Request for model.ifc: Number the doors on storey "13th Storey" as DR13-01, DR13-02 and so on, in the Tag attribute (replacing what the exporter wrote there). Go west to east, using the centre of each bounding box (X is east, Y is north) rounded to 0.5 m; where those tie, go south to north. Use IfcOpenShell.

First a look at what the model holds.

```python
import ifcopenshell
import ifcopenshell.util.element
import ifcopenshell.util.placement

model = ifcopenshell.open("model.ifc")
print(model.schema)
storey = next(s for s in model.by_type("IfcBuildingStorey") if s.Name == "13th Storey")
doors = [e for e in ifcopenshell.util.element.get_decomposition(storey) if e.is_a("IfcDoor")]
for e in sorted(doors, key=lambda e: e.id()):
    origin = ifcopenshell.util.placement.get_local_placement(e.ObjectPlacement)[:3, 3]
    print(e.id(), e.Tag, e.Name, origin.round(2) + 0.0, sep=" | ")
```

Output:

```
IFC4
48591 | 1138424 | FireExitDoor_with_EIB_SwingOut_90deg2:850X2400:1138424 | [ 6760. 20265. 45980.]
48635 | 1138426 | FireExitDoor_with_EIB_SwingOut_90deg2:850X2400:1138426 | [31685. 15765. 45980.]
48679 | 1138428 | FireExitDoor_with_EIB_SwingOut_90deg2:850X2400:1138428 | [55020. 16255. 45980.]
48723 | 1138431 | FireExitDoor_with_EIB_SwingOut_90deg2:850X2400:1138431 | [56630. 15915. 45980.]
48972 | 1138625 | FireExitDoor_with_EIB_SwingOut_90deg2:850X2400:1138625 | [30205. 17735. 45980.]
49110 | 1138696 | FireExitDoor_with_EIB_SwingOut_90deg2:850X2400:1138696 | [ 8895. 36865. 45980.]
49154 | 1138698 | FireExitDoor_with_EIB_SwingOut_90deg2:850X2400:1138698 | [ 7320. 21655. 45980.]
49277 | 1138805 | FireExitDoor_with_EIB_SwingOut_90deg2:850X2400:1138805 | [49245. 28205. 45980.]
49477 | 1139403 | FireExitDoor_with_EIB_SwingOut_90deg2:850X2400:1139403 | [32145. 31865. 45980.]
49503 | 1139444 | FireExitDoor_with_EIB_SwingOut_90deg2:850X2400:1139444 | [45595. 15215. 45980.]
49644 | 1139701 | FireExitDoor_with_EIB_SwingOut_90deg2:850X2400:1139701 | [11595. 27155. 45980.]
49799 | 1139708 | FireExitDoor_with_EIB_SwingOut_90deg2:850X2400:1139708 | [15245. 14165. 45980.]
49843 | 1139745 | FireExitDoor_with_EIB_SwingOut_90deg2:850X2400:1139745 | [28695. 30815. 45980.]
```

```python
import ifcopenshell
import ifcopenshell.geom
import ifcopenshell.util.element
import ifcopenshell.util.shape

model = ifcopenshell.open("model.ifc")
settings = ifcopenshell.geom.settings()
settings.set("use-world-coords", True)


def centre(element):
    shape = ifcopenshell.geom.create_shape(settings, element)
    return ifcopenshell.util.shape.get_bbox_centroid(shape.geometry)


storey = next(s for s in model.by_type("IfcBuildingStorey") if s.Name == "13th Storey")
doors = [e for e in ifcopenshell.util.element.get_decomposition(storey) if e.is_a("IfcDoor")]

# Insertion points can sit at a corner or the storey origin, so sort by the geometry (in metres).
centres = {e: centre(e) for e in doors}
doors.sort(key=lambda e: (round(centres[e][0] / 0.5), centres[e][1]))

for i, e in enumerate(doors, start=1):
    number = f"DR13-{i:02d}"
    e.Tag = number
    print(e.id(), number)

model.write("model-out.ifc")
```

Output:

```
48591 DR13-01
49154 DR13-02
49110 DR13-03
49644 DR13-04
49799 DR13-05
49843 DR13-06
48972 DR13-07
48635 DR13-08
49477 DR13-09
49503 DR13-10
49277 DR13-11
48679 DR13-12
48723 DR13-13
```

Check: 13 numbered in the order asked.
